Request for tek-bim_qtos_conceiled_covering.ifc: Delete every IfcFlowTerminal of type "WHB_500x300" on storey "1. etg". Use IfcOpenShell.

First a look at what the model holds.

```python
import ifcopenshell
import ifcopenshell.util.element

model = ifcopenshell.open("tek-bim_qtos_conceiled_covering.ifc")
print(model.schema)
storey = next(s for s in model.by_type("IfcBuildingStorey") if s.Name == "1. etg")
terminals = [e for e in ifcopenshell.util.element.get_decomposition(storey) if e.is_a("IfcFlowTerminal")]
seen = {}
for e in terminals:
    element_type = ifcopenshell.util.element.get_type(e)
    name = element_type.Name if element_type not in (None, e) else None
    seen[name] = seen.get(name, 0) + 1
for name, count in sorted(seen.items(), key=str):
    print(count, "x", name)
```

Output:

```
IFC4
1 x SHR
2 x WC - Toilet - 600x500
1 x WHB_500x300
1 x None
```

```python
import ifcopenshell
import ifcopenshell.api.root
import ifcopenshell.util.element

model = ifcopenshell.open("tek-bim_qtos_conceiled_covering.ifc")

storey = next(s for s in model.by_type("IfcBuildingStorey") if s.Name == "1. etg")
terminals = [e for e in ifcopenshell.util.element.get_decomposition(storey) if e.is_a("IfcFlowTerminal")]
targets = [e for e in terminals if (t := ifcopenshell.util.element.get_type(e)) not in (None, e) and t.Name == "WHB_500x300"]

for e in targets:
    ifcopenshell.api.root.remove_product(model, product=e)
print(len(targets), "removed")

model.write("tek-bim_qtos_conceiled_covering_v2.ifc")
```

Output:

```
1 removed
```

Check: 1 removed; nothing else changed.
